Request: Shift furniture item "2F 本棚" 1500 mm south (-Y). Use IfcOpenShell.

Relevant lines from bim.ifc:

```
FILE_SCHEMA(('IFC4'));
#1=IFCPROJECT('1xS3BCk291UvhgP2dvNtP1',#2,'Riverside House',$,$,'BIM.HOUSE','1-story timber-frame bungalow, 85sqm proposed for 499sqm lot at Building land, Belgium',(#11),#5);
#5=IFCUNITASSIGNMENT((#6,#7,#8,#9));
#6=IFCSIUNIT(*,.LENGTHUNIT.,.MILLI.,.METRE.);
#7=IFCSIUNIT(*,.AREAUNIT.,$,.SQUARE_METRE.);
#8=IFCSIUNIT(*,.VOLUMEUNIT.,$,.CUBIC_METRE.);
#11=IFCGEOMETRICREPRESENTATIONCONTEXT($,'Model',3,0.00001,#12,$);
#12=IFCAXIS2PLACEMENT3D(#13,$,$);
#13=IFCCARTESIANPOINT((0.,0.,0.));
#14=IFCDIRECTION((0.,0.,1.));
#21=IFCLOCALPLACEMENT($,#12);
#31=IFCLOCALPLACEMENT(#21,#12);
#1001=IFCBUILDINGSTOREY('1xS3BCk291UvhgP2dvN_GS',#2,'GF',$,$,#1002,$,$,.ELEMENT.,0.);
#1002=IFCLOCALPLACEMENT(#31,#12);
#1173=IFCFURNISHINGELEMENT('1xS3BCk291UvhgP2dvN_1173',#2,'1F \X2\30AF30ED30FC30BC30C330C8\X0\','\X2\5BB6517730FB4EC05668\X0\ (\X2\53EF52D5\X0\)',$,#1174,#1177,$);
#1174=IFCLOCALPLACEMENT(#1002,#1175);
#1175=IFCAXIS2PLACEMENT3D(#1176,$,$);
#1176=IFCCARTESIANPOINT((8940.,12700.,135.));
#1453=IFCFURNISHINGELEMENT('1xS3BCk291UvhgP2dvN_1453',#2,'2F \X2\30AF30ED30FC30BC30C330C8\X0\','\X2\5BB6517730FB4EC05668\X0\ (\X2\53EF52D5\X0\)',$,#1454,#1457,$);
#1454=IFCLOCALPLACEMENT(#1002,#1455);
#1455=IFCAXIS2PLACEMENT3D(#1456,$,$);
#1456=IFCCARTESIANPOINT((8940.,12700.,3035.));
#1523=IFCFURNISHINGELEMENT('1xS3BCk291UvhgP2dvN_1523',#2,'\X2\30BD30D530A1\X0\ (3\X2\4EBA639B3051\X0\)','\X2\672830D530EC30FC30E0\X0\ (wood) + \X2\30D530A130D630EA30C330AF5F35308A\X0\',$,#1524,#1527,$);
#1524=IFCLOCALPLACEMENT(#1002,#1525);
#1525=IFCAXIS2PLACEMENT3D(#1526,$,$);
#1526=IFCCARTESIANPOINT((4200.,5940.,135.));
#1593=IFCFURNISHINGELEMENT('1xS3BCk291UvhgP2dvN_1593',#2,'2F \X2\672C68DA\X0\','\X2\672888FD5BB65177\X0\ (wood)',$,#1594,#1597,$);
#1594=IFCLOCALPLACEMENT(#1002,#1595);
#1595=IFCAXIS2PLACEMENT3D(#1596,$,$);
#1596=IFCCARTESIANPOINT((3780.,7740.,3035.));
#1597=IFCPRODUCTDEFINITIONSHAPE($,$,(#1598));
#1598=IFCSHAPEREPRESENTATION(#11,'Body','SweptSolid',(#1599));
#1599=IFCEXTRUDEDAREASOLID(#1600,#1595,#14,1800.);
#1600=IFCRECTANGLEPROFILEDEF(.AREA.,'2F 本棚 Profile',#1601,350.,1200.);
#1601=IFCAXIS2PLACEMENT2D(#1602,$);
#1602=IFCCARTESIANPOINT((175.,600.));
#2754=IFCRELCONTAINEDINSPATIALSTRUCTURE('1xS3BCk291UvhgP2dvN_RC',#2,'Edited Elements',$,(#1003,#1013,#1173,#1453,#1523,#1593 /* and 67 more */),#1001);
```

```python
import ifcopenshell
import ifcopenshell.api.geometry
import ifcopenshell.util.placement

model = ifcopenshell.open("bim.ifc")

item = model.by_guid("1xS3BCk291UvhgP2dvN_1593")
matrix = ifcopenshell.util.placement.get_local_placement(item.ObjectPlacement)
matrix[1, 3] -= 1500.0
ifcopenshell.api.geometry.edit_object_placement(model, product=item, matrix=matrix, is_si=False)

print(ifcopenshell.util.placement.get_local_placement(item.ObjectPlacement).round(3) + 0.0)

model.write("bim_edited.ifc")
```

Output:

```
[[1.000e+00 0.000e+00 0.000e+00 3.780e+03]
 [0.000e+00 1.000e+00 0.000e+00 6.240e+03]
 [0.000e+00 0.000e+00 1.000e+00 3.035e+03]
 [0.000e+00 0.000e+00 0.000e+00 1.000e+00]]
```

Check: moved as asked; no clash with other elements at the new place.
